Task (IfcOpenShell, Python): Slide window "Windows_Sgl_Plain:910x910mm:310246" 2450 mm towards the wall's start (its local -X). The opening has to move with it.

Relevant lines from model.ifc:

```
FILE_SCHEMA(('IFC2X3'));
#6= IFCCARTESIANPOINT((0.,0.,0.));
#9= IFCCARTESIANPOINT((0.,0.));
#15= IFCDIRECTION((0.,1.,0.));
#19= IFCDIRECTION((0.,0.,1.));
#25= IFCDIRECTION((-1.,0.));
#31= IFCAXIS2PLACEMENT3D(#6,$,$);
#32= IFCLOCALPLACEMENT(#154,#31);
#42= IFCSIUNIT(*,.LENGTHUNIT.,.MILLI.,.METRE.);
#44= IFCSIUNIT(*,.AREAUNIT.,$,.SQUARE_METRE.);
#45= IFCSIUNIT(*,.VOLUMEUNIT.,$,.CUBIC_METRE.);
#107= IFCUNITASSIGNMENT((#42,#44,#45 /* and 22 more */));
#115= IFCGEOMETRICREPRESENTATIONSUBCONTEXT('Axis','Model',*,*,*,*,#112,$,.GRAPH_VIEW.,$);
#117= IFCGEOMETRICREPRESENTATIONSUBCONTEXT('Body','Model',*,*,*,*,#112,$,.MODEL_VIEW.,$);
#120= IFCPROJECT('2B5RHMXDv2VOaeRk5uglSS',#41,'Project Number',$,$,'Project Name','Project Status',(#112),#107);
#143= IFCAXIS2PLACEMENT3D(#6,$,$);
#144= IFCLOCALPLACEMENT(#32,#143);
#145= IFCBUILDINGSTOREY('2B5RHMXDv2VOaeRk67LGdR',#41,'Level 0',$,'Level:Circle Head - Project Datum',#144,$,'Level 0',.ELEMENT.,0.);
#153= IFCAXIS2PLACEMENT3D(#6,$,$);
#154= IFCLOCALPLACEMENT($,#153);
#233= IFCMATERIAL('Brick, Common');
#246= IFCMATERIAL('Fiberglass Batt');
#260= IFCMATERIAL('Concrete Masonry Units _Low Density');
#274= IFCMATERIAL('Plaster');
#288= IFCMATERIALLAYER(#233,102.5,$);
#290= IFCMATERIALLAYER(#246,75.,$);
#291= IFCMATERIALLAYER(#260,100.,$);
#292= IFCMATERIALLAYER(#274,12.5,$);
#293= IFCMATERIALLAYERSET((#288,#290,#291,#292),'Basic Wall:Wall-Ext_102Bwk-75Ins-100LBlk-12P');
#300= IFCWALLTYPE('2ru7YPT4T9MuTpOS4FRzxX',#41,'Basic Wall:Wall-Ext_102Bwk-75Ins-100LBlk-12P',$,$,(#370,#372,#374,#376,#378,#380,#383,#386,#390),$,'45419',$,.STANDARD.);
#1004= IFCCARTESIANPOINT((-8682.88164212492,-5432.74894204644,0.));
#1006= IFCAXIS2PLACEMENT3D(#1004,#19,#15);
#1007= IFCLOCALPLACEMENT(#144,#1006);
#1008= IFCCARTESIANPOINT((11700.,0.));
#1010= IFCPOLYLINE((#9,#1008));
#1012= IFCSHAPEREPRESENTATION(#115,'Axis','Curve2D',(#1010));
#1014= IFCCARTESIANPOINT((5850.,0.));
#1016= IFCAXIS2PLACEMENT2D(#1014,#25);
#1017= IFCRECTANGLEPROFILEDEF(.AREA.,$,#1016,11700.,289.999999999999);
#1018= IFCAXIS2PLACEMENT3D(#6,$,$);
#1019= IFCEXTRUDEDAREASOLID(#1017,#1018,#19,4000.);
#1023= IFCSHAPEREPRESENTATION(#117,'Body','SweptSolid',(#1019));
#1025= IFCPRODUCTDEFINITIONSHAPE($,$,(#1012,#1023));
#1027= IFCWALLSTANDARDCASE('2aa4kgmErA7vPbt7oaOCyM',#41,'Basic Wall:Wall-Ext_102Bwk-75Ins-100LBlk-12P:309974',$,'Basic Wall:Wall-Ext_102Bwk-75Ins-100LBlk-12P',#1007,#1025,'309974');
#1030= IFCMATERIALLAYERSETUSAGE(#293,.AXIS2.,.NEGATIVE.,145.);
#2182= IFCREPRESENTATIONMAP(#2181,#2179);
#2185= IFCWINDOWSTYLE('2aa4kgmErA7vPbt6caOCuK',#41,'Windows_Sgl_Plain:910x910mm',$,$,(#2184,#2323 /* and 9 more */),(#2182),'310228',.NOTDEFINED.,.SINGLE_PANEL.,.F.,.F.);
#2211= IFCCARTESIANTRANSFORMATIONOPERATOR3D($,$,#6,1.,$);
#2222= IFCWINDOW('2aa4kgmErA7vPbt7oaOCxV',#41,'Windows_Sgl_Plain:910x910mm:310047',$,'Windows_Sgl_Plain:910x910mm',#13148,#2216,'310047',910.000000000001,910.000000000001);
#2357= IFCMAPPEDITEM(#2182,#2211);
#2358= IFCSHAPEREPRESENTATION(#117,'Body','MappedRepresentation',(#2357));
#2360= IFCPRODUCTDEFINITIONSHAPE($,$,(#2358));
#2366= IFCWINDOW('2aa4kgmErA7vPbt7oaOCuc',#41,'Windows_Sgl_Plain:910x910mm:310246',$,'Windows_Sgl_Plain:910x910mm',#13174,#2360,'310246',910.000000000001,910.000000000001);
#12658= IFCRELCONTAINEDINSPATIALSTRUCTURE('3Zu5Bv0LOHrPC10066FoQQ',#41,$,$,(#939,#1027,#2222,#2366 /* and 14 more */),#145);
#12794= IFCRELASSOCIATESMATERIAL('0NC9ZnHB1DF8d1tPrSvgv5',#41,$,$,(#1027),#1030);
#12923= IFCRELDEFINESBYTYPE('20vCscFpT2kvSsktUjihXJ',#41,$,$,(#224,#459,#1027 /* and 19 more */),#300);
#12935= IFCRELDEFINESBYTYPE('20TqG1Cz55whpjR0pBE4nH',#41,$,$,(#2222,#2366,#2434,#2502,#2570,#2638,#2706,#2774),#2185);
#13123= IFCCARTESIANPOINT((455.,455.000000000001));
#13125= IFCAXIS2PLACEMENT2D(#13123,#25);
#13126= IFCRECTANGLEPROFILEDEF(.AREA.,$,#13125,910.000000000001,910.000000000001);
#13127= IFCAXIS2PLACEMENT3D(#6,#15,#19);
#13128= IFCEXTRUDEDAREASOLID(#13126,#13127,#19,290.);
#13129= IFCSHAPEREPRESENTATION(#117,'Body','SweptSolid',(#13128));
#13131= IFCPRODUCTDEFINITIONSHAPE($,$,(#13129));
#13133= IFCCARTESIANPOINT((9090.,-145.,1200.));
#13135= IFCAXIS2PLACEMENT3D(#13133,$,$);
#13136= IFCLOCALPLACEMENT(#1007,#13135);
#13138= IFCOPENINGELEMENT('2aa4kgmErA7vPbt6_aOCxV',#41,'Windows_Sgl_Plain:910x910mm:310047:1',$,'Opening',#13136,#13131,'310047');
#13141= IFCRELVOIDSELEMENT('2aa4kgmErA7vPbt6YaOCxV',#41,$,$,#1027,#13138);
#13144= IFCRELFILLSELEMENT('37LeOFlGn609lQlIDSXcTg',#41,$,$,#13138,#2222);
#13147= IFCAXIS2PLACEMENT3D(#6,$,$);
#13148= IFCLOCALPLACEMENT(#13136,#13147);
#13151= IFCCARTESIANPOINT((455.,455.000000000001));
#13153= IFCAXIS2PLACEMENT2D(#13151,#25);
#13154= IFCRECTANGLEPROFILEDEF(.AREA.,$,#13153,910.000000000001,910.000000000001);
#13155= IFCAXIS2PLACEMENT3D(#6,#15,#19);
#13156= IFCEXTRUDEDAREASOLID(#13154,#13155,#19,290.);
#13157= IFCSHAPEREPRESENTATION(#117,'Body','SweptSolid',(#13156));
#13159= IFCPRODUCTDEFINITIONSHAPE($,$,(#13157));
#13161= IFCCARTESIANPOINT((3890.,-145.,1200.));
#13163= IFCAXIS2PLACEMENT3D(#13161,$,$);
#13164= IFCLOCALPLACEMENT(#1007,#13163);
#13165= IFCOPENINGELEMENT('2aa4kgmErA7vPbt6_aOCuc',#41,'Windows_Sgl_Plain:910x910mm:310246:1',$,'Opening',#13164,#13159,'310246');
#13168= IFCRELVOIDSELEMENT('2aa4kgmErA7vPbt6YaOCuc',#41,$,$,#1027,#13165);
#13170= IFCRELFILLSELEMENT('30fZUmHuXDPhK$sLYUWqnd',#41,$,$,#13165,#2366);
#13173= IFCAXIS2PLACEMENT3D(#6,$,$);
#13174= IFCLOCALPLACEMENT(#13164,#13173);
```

```python
import ifcopenshell
import ifcopenshell.api.geometry
import ifcopenshell.util.placement
import ifcopenshell.util.unit

model = ifcopenshell.open("model.ifc")
unit_scale = ifcopenshell.util.unit.calculate_unit_scale(model)

window = model.by_guid("2aa4kgmErA7vPbt7oaOCuc")
opening = window.FillsVoids[0].RelatingOpeningElement
wall = opening.VoidsElements[0].RelatingBuildingElement

wall_matrix = ifcopenshell.util.placement.get_local_placement(wall.ObjectPlacement)
shift = wall_matrix[:3, 0] * -2.45 / unit_scale
before = ifcopenshell.util.placement.get_local_placement(window.ObjectPlacement)[:3, 3].copy()

# The window is placed relative to its opening, so it follows when the opening moves.
matrix = ifcopenshell.util.placement.get_local_placement(opening.ObjectPlacement)
matrix[:3, 3] += shift
ifcopenshell.api.geometry.edit_object_placement(
    model, product=opening, matrix=matrix, is_si=False, should_transform_children=True
)

after = ifcopenshell.util.placement.get_local_placement(window.ObjectPlacement)[:3, 3]
print("window moved by", (after - before).round(3) + 0.0)

model.write("model-out.ifc")
```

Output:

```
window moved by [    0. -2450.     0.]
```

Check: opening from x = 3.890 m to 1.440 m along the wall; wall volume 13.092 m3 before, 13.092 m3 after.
